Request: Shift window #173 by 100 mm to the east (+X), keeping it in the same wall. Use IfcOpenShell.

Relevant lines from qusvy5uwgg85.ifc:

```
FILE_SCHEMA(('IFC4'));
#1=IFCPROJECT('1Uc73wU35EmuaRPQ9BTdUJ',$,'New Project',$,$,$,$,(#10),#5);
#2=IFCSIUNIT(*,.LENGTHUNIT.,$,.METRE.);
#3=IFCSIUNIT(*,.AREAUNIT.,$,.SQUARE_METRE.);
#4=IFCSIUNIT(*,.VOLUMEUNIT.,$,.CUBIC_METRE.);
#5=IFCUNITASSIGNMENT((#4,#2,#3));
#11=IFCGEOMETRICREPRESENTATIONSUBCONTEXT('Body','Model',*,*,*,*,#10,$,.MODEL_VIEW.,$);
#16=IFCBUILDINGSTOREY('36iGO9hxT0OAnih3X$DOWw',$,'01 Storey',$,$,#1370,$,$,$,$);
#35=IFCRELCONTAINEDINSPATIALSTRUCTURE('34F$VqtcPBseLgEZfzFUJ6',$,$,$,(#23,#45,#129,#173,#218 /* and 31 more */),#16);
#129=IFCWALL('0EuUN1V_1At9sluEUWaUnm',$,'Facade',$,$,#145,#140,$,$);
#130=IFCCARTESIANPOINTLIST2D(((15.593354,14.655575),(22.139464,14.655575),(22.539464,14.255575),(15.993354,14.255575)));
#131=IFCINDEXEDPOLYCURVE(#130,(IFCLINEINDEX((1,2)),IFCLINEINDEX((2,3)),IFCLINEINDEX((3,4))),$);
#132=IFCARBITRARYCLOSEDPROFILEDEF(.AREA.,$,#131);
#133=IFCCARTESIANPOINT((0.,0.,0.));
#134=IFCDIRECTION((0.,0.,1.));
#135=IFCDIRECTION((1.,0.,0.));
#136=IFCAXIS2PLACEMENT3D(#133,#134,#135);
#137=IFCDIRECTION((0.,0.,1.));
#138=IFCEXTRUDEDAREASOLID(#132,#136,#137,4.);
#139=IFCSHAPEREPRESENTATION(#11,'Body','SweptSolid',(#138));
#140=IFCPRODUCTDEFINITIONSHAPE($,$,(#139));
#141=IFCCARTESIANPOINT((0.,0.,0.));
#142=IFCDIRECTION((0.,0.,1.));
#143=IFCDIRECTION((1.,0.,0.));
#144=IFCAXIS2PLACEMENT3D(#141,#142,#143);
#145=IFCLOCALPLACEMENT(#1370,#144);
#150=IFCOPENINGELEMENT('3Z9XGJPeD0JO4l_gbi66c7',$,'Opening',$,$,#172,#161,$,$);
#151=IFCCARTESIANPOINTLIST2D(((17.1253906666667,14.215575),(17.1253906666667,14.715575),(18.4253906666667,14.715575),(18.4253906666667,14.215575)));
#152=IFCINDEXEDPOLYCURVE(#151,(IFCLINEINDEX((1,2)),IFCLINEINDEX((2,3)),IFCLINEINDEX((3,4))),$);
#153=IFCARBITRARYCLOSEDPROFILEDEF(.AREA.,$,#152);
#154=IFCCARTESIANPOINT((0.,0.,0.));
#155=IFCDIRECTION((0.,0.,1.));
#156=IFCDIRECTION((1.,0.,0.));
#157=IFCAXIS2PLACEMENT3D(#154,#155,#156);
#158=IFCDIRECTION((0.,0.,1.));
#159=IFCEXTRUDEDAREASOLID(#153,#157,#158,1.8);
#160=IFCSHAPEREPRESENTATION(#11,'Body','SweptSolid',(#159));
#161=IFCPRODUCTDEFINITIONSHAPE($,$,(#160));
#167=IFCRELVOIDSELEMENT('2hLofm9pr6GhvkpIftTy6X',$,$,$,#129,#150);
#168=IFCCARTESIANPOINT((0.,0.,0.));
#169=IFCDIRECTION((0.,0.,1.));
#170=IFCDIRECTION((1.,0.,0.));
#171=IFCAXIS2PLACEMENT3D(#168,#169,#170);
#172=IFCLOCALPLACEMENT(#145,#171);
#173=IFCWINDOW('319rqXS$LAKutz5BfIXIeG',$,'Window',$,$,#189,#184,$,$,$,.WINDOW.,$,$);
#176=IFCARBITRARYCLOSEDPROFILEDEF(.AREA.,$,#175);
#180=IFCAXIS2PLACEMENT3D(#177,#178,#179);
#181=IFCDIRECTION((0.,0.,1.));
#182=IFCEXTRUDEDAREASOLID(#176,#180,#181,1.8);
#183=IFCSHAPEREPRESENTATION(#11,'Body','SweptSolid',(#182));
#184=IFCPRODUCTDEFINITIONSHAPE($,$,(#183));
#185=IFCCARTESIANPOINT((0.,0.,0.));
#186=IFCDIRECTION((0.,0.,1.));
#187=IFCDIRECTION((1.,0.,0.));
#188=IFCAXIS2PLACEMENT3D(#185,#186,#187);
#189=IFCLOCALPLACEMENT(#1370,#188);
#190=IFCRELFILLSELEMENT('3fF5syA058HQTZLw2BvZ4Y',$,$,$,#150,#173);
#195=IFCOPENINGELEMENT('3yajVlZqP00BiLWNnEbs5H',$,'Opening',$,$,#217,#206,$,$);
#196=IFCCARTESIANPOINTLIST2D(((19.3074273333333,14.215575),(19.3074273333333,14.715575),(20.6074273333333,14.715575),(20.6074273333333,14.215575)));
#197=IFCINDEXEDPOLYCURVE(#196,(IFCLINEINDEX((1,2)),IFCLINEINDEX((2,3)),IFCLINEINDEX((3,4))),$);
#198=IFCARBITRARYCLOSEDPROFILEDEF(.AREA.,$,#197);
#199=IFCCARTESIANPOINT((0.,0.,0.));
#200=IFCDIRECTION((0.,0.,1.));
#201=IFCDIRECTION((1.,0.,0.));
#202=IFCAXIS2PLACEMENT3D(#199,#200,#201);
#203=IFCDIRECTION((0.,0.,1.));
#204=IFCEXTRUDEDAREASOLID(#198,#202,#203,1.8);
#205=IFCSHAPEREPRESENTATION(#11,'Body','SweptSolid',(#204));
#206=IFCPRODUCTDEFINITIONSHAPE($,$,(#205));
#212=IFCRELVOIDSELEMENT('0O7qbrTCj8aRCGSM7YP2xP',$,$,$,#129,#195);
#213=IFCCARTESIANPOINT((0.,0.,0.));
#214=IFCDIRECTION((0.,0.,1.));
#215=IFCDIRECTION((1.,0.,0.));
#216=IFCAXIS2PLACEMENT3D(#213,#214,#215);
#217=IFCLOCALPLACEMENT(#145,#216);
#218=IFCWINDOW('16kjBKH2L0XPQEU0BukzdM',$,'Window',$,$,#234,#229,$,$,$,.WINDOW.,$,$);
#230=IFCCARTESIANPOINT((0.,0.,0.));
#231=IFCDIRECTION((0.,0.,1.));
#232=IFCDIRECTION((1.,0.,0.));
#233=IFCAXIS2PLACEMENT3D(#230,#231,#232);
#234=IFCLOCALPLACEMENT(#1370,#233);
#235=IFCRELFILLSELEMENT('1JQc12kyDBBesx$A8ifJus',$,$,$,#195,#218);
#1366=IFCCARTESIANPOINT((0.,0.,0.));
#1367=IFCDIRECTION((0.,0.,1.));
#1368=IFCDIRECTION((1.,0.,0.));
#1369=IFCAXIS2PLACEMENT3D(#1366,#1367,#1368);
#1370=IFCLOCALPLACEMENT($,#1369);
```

```python
import ifcopenshell
import ifcopenshell.api.geometry
import ifcopenshell.util.placement

model = ifcopenshell.open("qusvy5uwgg85.ifc")

window = model.by_id(173)
opening = window.FillsVoids[0].RelatingOpeningElement
wall = opening.VoidsElements[0].RelatingBuildingElement

wall_matrix = ifcopenshell.util.placement.get_local_placement(wall.ObjectPlacement)
shift = wall_matrix[:3, 0] * 0.1
before = ifcopenshell.util.placement.get_local_placement(window.ObjectPlacement)[:3, 3].copy()

# The window is not placed relative to its opening, so move both.
for product in (opening, window):
    matrix = ifcopenshell.util.placement.get_local_placement(product.ObjectPlacement)
    matrix[:3, 3] += shift
    ifcopenshell.api.geometry.edit_object_placement(model, product=product, matrix=matrix, is_si=False)

after = ifcopenshell.util.placement.get_local_placement(window.ObjectPlacement)[:3, 3]
print("window moved by", (after - before).round(3) + 0.0)

model.write("qusvy5uwgg85_rev.ifc")
```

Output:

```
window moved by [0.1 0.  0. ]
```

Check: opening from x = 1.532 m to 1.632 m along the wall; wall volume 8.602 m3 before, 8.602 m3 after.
